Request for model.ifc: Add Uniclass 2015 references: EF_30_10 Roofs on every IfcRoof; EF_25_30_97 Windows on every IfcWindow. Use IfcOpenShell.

First a look at what the model holds.

```python
import ifcopenshell

model = ifcopenshell.open("model.ifc")
print(model.schema)
print("classifications:", [c.Name for c in model.by_type("IfcClassification")])
for ifc_class in ("IfcDoor", "IfcRoof", "IfcStair", "IfcWall", "IfcWindow"):
    print(ifc_class, len(model.by_type(ifc_class)))
```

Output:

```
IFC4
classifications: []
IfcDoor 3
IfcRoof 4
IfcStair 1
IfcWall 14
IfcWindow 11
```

```python
import ifcopenshell
import ifcopenshell.api.classification

model = ifcopenshell.open("model.ifc")

system = ifcopenshell.api.classification.add_classification(model, classification="Uniclass 2015")

codes = {
    "IfcRoof": ("EF_30_10", "Roofs"),
    "IfcWindow": ("EF_25_30_97", "Windows"),
}
for ifc_class, (code, name) in codes.items():
    products = model.by_type(ifc_class)
    ifcopenshell.api.classification.add_reference(
        model, products=products, classification=system, identification=code, name=name
    )
    print(code, len(products))

model.write("model_edited.ifc")
```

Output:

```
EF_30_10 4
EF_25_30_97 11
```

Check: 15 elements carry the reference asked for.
